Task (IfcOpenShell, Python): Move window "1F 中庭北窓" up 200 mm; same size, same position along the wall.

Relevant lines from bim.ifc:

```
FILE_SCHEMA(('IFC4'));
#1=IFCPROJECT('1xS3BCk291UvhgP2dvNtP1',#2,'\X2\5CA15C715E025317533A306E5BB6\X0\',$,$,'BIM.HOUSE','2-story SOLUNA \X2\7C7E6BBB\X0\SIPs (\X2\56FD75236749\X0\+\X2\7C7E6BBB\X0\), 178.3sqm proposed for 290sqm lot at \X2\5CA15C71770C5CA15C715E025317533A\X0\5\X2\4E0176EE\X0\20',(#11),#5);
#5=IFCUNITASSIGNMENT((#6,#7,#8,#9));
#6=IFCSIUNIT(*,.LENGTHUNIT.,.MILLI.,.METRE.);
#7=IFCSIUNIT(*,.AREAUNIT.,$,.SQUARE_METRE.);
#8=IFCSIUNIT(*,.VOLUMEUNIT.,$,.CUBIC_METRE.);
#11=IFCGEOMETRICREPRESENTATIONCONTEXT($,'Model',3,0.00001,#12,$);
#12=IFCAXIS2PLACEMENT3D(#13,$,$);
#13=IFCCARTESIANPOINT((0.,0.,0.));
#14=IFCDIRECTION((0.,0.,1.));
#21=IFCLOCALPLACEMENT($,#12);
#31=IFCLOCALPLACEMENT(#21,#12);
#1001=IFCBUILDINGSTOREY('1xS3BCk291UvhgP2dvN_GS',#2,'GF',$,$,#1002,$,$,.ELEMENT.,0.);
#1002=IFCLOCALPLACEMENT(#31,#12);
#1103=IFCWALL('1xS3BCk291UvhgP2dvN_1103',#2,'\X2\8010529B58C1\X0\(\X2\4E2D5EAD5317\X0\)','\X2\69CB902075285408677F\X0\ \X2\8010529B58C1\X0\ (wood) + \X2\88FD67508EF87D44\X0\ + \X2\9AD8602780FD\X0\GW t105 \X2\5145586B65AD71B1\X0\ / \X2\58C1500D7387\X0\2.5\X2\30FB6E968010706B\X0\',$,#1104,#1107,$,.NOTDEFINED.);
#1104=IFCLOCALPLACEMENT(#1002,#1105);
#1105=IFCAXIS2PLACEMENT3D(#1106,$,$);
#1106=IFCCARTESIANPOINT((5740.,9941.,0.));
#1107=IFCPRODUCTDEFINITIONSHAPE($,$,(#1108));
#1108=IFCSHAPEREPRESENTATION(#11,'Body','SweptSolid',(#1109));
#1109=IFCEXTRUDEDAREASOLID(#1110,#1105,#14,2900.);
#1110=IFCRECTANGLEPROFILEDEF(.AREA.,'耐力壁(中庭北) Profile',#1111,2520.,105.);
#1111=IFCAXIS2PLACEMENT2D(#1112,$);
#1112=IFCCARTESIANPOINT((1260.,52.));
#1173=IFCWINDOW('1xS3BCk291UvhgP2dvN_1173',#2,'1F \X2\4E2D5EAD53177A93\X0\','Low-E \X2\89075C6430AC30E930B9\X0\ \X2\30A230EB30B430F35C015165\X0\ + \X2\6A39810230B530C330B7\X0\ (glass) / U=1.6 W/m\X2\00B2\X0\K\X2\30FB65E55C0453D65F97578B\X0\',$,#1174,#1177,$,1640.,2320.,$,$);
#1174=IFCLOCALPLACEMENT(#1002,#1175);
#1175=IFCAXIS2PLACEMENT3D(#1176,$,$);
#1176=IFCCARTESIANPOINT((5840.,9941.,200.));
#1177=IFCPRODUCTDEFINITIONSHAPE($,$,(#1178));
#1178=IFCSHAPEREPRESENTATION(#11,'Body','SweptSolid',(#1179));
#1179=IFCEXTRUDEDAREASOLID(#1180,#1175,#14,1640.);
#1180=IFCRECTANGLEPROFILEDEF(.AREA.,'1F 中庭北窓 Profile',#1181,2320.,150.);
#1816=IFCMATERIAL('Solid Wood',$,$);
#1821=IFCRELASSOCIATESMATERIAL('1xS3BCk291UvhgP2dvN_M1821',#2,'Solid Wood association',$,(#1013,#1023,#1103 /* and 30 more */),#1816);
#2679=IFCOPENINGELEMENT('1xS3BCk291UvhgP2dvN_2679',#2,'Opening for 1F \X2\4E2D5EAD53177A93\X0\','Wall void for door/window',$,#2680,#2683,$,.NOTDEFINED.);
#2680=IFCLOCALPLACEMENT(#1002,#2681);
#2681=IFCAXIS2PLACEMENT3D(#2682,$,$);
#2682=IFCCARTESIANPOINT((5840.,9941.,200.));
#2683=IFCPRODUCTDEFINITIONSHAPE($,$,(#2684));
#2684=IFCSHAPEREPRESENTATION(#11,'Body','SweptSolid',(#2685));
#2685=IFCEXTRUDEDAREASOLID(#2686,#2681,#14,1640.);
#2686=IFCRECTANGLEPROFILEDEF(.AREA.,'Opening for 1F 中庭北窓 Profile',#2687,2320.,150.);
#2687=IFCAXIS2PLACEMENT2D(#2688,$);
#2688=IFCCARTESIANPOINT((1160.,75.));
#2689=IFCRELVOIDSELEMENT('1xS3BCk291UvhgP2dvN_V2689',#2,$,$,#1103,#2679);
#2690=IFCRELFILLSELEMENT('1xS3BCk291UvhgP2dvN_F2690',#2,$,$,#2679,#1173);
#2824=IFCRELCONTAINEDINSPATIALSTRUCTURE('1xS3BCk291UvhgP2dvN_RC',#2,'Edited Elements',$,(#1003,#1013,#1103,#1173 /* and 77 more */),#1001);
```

```python
import numpy as np
import ifcopenshell
import ifcopenshell.api.geometry
import ifcopenshell.util.placement
import ifcopenshell.util.unit

model = ifcopenshell.open("bim.ifc")
unit_scale = ifcopenshell.util.unit.calculate_unit_scale(model)

window = model.by_guid("1xS3BCk291UvhgP2dvN_1173")
opening = window.FillsVoids[0].RelatingOpeningElement
dz = 0.2 / unit_scale

shift = np.array([0.0, 0.0, dz])
# The window is not placed relative to its opening, so move both.
for product in (opening, window):
    matrix = ifcopenshell.util.placement.get_local_placement(product.ObjectPlacement)
    matrix[:3, 3] += shift
    ifcopenshell.api.geometry.edit_object_placement(model, product=product, matrix=matrix, is_si=False)

print(f"moved by {dz * unit_scale:+.3f} m")

model.write("bim_updated.ifc")
```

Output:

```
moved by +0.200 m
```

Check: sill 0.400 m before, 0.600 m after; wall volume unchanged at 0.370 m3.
